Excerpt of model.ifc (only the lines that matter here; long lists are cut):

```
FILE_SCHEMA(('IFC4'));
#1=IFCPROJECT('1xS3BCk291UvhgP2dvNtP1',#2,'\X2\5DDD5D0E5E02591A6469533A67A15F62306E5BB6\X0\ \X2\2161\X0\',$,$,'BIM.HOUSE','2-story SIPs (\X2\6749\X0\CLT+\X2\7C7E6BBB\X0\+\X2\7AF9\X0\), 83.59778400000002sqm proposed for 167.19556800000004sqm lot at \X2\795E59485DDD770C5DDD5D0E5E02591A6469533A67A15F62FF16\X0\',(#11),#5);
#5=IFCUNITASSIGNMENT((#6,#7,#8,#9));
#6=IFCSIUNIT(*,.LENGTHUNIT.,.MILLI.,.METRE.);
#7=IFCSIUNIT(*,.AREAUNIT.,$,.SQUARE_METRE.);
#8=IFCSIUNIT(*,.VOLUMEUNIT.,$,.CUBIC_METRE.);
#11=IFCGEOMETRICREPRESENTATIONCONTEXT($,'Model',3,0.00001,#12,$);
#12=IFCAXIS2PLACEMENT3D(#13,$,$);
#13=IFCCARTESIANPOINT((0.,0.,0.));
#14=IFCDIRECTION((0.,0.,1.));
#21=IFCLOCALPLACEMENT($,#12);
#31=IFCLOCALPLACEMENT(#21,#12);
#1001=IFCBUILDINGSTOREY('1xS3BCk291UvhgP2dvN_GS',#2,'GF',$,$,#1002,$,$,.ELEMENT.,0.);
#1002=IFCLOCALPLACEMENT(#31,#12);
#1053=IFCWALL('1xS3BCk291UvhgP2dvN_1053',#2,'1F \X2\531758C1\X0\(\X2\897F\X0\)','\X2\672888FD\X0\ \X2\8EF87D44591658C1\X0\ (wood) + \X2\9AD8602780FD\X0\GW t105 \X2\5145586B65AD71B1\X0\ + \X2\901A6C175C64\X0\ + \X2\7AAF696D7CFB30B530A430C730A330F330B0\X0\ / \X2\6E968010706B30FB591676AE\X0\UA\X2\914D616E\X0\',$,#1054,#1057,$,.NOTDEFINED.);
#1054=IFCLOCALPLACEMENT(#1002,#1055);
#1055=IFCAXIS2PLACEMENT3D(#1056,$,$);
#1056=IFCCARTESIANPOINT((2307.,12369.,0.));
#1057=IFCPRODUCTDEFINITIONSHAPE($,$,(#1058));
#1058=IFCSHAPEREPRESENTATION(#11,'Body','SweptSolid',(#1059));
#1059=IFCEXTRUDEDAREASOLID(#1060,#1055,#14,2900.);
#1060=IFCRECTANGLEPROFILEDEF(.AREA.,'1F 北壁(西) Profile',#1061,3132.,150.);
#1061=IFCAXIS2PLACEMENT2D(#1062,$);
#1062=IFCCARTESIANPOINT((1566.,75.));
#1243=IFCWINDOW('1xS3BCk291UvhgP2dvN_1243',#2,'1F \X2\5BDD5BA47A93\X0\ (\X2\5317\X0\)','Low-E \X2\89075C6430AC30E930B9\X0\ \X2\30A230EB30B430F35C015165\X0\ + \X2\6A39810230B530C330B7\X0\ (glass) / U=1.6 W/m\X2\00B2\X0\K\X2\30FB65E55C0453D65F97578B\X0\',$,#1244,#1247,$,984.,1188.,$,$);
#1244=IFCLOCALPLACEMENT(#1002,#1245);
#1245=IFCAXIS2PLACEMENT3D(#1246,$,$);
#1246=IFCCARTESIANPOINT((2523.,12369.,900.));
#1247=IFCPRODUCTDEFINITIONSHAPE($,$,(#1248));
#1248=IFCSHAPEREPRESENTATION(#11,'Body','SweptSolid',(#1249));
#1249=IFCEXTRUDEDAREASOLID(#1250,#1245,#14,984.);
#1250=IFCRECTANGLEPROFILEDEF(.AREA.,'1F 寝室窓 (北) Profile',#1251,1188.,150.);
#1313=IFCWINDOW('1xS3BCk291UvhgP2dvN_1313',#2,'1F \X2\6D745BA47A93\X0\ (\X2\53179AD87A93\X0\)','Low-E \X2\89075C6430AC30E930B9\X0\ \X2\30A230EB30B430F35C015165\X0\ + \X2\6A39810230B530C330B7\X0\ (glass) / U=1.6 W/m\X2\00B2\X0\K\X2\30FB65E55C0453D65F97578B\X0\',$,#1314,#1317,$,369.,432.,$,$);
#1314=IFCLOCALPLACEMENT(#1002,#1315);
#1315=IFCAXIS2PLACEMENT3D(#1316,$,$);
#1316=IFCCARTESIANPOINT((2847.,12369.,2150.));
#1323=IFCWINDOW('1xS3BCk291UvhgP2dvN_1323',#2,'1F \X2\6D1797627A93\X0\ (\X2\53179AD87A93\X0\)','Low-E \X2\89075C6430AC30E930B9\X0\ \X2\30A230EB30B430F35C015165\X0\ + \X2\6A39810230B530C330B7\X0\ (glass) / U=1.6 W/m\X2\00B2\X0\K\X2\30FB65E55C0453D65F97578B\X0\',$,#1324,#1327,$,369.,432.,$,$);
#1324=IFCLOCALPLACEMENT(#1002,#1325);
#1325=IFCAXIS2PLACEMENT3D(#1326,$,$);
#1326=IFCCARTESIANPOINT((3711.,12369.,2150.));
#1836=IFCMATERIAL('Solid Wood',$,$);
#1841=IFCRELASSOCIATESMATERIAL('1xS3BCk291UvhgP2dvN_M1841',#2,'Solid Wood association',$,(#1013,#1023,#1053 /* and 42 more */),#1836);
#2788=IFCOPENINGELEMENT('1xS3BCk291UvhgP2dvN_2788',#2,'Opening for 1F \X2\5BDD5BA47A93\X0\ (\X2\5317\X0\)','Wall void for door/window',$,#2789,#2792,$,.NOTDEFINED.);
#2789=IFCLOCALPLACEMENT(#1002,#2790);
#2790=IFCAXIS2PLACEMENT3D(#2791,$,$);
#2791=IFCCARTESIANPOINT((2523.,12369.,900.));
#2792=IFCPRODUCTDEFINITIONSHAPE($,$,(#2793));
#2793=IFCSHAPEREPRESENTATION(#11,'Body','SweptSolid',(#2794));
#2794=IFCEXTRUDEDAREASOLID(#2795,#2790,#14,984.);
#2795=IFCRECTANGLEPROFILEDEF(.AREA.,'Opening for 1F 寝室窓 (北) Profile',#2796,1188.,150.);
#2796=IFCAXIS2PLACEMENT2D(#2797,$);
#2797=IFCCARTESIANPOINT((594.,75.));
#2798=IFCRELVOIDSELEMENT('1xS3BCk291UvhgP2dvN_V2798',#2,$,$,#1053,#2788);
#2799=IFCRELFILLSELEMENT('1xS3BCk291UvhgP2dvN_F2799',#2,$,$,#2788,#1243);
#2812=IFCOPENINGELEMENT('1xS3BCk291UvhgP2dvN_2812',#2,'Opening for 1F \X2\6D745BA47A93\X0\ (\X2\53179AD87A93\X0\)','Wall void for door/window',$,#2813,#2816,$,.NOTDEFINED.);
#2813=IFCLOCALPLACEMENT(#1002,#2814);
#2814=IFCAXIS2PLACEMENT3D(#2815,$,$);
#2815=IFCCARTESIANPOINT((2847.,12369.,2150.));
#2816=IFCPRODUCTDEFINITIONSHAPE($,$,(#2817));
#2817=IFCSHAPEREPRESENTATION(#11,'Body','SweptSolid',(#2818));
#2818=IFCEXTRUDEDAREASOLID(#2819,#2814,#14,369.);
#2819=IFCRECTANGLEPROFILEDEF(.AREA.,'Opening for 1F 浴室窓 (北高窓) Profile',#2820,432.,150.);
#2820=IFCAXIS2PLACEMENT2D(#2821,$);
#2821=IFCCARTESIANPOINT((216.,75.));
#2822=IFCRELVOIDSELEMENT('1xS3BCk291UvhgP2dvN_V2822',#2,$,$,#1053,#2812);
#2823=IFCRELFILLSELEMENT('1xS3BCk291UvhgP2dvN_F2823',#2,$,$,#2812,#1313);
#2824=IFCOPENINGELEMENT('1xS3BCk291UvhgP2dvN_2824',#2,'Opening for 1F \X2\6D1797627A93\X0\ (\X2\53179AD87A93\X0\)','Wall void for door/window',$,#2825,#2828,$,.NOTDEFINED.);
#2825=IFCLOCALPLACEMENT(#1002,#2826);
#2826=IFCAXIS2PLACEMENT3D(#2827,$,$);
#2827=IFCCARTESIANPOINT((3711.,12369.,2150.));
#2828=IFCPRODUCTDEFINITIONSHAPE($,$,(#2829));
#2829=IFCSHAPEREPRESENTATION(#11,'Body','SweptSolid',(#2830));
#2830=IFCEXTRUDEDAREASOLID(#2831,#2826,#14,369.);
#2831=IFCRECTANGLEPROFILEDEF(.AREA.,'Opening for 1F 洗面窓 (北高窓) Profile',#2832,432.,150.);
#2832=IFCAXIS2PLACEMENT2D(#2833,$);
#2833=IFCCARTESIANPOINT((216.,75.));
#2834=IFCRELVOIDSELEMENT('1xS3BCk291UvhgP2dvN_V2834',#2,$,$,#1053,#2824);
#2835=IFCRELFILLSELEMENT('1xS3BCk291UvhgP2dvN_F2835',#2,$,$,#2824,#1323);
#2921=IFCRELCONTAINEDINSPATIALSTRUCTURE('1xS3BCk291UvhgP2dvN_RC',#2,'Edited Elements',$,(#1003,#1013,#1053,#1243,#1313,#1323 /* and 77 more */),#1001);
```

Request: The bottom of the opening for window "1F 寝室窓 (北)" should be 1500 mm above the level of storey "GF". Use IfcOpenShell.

```python
import numpy as np
import ifcopenshell
import ifcopenshell.api.geometry
import ifcopenshell.geom
import ifcopenshell.util.element
import ifcopenshell.util.placement
import ifcopenshell.util.shape
import ifcopenshell.util.unit

model = ifcopenshell.open("model.ifc")
unit_scale = ifcopenshell.util.unit.calculate_unit_scale(model)

window = model.by_guid("1xS3BCk291UvhgP2dvN_1243")
opening = window.FillsVoids[0].RelatingOpeningElement
storey = ifcopenshell.util.element.get_container(window, ifc_class="IfcBuildingStorey")
level = ifcopenshell.util.placement.get_local_placement(storey.ObjectPlacement)[2, 3]

# The opening's origin need not be at the sill, so measure its lowest point.
shape = ifcopenshell.geom.create_shape(ifcopenshell.geom.settings(), opening)
bottom = ifcopenshell.util.shape.get_shape_bottom_elevation(shape, shape.geometry) / unit_scale
dz = level + 1.5 / unit_scale - bottom

shift = np.array([0.0, 0.0, dz])
# The window is not placed relative to its opening, so move both.
for product in (opening, window):
    matrix = ifcopenshell.util.placement.get_local_placement(product.ObjectPlacement)
    matrix[:3, 3] += shift
    ifcopenshell.api.geometry.edit_object_placement(model, product=product, matrix=matrix, is_si=False)

print(f"moved by {dz * unit_scale:+.3f} m")

model.write("model_edited.ifc")
```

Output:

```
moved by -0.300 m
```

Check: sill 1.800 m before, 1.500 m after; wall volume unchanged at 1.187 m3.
